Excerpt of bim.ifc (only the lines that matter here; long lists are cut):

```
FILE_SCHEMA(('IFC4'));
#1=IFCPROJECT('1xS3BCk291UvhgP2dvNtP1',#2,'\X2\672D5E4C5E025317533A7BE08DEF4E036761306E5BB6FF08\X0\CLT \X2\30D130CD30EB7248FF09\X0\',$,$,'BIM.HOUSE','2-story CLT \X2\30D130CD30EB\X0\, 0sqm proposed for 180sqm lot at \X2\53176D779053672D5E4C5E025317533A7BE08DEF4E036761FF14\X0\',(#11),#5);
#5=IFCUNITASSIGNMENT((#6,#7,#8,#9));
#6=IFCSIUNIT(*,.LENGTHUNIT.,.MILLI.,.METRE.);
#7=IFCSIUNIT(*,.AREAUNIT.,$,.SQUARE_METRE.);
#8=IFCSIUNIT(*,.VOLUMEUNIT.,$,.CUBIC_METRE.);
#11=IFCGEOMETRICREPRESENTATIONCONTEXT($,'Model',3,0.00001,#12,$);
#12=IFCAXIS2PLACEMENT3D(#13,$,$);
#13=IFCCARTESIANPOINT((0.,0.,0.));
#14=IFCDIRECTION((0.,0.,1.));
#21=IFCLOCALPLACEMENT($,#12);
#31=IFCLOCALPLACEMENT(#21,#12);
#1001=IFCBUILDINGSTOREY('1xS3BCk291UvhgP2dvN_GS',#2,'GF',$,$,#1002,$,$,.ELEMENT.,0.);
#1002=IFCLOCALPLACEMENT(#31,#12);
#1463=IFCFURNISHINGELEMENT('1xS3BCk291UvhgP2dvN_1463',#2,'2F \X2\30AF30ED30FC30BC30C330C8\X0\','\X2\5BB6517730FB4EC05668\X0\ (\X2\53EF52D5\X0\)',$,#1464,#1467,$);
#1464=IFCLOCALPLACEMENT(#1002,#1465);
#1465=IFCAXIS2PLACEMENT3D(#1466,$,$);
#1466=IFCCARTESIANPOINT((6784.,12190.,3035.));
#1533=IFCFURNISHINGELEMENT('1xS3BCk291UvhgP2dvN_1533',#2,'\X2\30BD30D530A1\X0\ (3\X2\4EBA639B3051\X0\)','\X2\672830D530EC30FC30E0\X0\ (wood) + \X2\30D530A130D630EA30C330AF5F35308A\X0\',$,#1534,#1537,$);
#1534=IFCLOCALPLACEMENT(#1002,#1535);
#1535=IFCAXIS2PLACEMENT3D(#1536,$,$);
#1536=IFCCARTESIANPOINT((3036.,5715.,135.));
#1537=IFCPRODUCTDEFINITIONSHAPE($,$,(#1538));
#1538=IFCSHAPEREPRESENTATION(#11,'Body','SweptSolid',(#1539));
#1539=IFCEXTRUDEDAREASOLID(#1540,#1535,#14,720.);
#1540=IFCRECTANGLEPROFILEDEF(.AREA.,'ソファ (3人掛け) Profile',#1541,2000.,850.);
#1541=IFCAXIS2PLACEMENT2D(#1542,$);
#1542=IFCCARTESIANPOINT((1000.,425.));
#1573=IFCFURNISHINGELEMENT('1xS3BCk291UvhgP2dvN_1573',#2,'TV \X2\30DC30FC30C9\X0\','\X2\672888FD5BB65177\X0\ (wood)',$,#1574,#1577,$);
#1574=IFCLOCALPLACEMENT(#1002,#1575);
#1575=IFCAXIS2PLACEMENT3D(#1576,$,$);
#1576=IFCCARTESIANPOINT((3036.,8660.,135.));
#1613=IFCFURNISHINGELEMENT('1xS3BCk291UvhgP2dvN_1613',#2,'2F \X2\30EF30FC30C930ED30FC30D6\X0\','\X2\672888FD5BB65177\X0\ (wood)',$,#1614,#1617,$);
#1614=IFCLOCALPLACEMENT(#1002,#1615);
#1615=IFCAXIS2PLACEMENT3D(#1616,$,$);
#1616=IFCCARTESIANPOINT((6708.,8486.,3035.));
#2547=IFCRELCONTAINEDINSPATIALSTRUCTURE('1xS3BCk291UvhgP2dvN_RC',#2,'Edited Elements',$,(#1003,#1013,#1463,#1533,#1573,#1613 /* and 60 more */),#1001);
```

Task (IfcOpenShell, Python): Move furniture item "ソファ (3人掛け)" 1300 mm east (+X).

```python
import ifcopenshell
import ifcopenshell.api.geometry
import ifcopenshell.util.placement
import ifcopenshell.util.unit

model = ifcopenshell.open("bim.ifc")
unit_scale = ifcopenshell.util.unit.calculate_unit_scale(model)

item = model.by_guid("1xS3BCk291UvhgP2dvN_1533")
matrix = ifcopenshell.util.placement.get_local_placement(item.ObjectPlacement)
matrix[0, 3] += 1.3 / unit_scale
ifcopenshell.api.geometry.edit_object_placement(model, product=item, matrix=matrix, is_si=False)

print(ifcopenshell.util.placement.get_local_placement(item.ObjectPlacement).round(3) + 0.0)

model.write("bim-out.ifc")
```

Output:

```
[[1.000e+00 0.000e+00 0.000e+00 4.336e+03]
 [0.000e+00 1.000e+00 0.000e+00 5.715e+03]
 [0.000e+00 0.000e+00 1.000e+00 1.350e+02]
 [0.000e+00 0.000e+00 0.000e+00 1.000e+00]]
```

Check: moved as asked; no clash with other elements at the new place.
